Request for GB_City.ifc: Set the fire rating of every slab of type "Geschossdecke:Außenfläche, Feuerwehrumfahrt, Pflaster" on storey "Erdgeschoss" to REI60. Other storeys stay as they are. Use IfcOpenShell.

First a look at what the model holds.

```python
import ifcopenshell
import ifcopenshell.util.element

model = ifcopenshell.open("GB_City.ifc")
print(model.schema)
storey = next(s for s in model.by_type("IfcBuildingStorey") if s.Name == "Erdgeschoss")
slabs = [e for e in ifcopenshell.util.element.get_decomposition(storey) if e.is_a("IfcSlab")]
seen = {}
for e in slabs:
    element_type = ifcopenshell.util.element.get_type(e)
    key = (element_type.Name if element_type != e and element_type else None, ifcopenshell.util.element.get_pset(e, "Pset_SlabCommon", "FireRating"))
    seen[key] = seen.get(key, 0) + 1
for (name, value), count in sorted(seen.items(), key=str):
    print(count, "x", name, "|", value)
```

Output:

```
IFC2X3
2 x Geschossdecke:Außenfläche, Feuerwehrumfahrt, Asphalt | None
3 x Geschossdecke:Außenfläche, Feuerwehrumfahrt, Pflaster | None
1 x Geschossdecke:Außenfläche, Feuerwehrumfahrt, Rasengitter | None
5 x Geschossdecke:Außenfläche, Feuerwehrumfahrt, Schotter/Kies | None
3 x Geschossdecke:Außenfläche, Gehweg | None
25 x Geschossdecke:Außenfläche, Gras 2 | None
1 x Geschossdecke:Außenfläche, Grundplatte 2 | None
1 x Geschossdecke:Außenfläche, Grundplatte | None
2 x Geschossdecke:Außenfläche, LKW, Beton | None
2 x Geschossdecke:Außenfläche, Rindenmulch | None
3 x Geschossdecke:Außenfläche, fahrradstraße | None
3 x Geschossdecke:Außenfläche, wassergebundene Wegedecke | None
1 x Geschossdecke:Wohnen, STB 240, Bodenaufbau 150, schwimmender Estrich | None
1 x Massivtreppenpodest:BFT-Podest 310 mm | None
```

```python
import ifcopenshell
import ifcopenshell.api.pset
import ifcopenshell.util.element

model = ifcopenshell.open("GB_City.ifc")

storey = next(s for s in model.by_type("IfcBuildingStorey") if s.Name == "Erdgeschoss")
slabs = [e for e in ifcopenshell.util.element.get_decomposition(storey) if e.is_a("IfcSlab")]

count = 0
for e in slabs:
    element_type = ifcopenshell.util.element.get_type(e)
    if element_type in (None, e) or element_type.Name != "Geschossdecke:Außenfläche, Feuerwehrumfahrt, Pflaster":
        continue
    # add_pset returns the element's existing set when there is one.
    pset = ifcopenshell.api.pset.add_pset(model, product=e, name="Pset_SlabCommon")
    ifcopenshell.api.pset.edit_pset(model, pset=pset, properties={"FireRating": "REI60"})
    count += 1

print(count, "slabs updated")

model.write("GB_City_updated.ifc")
```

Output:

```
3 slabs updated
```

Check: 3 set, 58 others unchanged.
